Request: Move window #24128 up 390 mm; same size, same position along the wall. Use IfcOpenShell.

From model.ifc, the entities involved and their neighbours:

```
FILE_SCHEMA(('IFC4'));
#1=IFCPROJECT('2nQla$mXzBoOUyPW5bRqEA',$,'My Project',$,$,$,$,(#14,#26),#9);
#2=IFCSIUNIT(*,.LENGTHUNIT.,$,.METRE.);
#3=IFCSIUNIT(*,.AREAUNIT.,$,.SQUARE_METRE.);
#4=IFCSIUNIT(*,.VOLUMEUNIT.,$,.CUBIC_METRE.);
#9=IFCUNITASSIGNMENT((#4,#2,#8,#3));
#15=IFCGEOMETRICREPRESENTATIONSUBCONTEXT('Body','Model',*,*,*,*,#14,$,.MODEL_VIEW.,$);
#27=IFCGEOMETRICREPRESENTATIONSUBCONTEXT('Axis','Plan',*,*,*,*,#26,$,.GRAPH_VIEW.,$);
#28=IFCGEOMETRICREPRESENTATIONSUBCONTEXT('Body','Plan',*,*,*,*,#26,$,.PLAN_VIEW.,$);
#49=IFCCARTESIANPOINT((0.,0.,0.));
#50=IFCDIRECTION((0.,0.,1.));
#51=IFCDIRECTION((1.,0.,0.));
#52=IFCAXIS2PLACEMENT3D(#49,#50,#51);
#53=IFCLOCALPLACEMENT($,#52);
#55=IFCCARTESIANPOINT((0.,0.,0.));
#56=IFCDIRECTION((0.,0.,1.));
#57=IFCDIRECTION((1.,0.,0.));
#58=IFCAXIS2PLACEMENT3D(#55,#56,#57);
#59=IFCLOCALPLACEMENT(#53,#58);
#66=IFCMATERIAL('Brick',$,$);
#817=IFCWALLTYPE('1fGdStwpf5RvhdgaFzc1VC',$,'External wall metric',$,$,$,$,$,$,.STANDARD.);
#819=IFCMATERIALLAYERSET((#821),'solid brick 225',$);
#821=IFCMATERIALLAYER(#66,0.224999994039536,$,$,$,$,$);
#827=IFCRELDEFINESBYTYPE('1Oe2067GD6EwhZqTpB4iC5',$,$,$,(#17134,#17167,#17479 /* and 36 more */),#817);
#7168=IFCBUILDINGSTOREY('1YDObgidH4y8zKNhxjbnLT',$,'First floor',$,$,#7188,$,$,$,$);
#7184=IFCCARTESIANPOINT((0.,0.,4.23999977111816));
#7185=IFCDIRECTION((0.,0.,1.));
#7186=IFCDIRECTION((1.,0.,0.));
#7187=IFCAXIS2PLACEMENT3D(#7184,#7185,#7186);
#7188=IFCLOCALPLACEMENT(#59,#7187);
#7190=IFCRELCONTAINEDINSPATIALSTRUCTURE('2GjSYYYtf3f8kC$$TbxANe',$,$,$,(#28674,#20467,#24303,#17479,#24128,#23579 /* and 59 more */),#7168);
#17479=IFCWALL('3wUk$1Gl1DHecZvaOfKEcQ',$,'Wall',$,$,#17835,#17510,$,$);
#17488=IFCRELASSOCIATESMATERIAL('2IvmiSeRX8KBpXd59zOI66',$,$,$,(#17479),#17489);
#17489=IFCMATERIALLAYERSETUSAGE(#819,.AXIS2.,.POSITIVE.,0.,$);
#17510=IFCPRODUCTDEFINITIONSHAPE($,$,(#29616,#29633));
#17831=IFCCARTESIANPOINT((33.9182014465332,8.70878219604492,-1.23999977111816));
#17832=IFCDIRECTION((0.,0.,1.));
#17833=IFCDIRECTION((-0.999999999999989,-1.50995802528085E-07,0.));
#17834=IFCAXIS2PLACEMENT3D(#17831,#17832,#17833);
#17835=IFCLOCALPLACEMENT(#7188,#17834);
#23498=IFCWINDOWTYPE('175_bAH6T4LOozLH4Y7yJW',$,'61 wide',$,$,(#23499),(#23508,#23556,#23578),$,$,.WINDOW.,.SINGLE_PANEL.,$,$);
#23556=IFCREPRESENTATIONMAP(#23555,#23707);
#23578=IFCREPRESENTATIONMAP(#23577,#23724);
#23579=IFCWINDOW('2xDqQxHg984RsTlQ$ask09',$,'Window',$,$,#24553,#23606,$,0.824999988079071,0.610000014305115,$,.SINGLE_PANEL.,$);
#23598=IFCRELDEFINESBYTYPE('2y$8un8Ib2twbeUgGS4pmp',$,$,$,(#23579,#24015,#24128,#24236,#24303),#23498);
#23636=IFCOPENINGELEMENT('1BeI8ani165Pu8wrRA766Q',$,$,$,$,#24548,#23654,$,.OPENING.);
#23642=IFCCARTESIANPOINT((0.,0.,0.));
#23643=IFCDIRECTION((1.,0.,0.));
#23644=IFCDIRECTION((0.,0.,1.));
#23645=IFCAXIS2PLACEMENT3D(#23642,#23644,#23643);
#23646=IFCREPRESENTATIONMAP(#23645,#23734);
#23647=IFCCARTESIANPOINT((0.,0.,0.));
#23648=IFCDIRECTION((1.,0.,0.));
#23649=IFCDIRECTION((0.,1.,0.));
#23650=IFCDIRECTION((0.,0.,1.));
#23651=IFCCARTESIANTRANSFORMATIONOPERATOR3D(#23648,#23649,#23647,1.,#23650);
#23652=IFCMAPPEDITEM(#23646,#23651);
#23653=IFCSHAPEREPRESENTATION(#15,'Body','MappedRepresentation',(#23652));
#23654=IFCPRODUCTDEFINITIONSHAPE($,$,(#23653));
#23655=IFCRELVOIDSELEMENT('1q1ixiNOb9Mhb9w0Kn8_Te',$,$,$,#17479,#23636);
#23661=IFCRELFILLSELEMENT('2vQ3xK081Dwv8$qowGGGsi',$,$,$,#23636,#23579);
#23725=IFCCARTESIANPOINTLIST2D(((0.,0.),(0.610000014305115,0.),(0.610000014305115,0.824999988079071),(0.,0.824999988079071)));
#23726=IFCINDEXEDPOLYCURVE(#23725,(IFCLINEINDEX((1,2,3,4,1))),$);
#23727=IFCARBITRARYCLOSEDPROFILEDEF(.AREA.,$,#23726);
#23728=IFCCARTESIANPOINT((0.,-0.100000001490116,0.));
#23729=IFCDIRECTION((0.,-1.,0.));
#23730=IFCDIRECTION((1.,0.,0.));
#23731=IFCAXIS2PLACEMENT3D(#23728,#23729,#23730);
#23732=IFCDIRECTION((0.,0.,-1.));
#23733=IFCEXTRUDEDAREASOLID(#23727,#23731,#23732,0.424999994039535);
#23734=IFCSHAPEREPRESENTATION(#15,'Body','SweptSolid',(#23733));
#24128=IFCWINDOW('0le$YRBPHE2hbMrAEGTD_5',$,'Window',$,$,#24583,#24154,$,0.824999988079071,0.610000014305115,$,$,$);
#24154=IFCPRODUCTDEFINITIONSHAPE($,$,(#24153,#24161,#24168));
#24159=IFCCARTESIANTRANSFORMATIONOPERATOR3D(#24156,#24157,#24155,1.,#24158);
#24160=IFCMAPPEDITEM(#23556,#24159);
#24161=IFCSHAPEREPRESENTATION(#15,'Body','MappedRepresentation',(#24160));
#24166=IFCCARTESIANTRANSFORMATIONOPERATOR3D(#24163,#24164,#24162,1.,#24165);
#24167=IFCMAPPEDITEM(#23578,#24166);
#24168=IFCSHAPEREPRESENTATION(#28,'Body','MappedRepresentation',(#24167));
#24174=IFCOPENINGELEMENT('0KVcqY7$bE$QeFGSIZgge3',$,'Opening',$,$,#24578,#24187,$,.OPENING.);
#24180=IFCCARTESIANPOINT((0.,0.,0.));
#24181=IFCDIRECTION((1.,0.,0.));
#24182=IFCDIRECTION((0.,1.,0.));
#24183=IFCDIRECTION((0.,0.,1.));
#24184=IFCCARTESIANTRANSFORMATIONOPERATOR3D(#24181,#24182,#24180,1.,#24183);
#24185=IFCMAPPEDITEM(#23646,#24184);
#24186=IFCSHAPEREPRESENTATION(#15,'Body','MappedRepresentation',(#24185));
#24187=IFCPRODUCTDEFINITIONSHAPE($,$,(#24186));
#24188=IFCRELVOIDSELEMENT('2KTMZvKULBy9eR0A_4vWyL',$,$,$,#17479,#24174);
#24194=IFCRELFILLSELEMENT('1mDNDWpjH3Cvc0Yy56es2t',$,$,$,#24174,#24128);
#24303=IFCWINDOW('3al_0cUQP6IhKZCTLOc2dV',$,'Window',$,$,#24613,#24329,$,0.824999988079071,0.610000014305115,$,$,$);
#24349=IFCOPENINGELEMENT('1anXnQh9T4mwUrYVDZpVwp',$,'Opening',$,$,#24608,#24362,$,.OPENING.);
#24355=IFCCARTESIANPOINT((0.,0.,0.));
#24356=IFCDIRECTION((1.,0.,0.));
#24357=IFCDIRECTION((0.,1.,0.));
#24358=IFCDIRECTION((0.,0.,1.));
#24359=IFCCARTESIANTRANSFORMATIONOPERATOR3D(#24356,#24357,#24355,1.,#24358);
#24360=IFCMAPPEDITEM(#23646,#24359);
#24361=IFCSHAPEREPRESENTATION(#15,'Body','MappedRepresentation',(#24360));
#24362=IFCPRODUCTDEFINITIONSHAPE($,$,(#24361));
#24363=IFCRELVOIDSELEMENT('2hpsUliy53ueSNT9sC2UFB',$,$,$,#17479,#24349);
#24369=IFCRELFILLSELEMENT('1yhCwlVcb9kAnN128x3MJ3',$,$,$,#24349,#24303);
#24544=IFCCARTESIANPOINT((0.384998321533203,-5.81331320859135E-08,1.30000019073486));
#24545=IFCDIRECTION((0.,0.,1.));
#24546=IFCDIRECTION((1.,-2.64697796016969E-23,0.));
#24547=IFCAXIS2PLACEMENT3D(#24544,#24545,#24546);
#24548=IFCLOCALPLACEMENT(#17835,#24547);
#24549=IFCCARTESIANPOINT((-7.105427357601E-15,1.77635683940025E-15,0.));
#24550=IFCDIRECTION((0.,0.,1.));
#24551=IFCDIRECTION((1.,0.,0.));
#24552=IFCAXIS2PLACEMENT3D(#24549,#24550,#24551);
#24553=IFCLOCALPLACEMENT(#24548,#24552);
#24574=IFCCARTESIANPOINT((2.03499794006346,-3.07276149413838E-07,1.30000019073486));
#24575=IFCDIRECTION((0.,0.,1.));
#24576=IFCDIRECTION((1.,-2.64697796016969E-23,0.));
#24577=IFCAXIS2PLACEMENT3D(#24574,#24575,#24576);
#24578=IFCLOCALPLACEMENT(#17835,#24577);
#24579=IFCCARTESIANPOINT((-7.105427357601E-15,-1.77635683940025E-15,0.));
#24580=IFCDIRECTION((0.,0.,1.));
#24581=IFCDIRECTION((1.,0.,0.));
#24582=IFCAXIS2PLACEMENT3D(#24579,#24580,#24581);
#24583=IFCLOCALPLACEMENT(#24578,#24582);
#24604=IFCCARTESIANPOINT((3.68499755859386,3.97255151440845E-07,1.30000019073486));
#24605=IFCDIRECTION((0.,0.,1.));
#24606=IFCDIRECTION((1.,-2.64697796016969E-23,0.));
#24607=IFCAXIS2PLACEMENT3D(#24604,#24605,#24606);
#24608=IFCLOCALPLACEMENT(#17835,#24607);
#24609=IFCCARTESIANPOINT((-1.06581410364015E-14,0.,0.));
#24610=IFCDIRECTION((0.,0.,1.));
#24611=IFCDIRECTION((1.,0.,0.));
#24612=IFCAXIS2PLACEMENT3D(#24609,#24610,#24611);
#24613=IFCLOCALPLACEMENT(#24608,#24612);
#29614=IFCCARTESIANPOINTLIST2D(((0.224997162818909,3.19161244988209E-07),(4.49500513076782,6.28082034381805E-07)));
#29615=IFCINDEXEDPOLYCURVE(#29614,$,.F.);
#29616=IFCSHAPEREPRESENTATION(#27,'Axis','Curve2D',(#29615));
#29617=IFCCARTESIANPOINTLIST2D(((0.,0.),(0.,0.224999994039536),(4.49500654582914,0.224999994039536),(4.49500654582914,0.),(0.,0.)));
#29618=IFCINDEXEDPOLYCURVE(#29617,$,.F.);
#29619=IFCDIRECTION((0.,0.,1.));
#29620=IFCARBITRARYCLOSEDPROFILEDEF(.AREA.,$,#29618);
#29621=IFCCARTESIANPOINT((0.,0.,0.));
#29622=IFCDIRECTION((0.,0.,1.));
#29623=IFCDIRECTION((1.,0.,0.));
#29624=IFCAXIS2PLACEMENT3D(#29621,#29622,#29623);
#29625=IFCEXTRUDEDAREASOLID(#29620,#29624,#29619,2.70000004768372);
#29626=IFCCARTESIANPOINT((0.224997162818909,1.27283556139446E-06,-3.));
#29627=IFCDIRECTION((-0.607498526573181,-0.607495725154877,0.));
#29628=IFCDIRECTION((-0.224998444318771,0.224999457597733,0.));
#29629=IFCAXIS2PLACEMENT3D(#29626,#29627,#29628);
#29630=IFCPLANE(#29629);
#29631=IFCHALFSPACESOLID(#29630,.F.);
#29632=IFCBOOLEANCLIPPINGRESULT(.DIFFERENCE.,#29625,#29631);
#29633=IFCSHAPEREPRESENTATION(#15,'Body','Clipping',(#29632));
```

```python
import numpy as np
import ifcopenshell
import ifcopenshell.api.geometry
import ifcopenshell.util.placement
import ifcopenshell.util.unit

model = ifcopenshell.open("model.ifc")
unit_scale = ifcopenshell.util.unit.calculate_unit_scale(model)

window = model.by_guid("0le$YRBPHE2hbMrAEGTD_5")
opening = window.FillsVoids[0].RelatingOpeningElement
dz = 0.39 / unit_scale

shift = np.array([0.0, 0.0, dz])
# The window is placed relative to its opening, so it follows when the opening moves.
matrix = ifcopenshell.util.placement.get_local_placement(opening.ObjectPlacement)
matrix[:3, 3] += shift
ifcopenshell.api.geometry.edit_object_placement(
    model, product=opening, matrix=matrix, is_si=False, should_transform_children=True
)

print(f"moved by {dz * unit_scale:+.3f} m")

model.write("model_edited.ifc")
```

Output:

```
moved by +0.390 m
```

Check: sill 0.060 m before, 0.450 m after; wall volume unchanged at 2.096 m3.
